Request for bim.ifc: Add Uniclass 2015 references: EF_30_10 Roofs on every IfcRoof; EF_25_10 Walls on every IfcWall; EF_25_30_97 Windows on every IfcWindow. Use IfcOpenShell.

First a look at what the model holds.

```python
import ifcopenshell

model = ifcopenshell.open("bim.ifc")
print(model.schema)
print("classifications:", [c.Name for c in model.by_type("IfcClassification")])
for ifc_class in ("IfcDoor", "IfcRoof", "IfcStair", "IfcWall", "IfcWindow"):
    print(ifc_class, len(model.by_type(ifc_class)))
```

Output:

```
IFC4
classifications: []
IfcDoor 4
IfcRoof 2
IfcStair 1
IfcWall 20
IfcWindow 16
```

```python
import ifcopenshell
import ifcopenshell.api.classification

model = ifcopenshell.open("bim.ifc")

system = ifcopenshell.api.classification.add_classification(model, classification="Uniclass 2015")

codes = {
    "IfcRoof": ("EF_30_10", "Roofs"),
    "IfcWall": ("EF_25_10", "Walls"),
    "IfcWindow": ("EF_25_30_97", "Windows"),
}
for ifc_class, (code, name) in codes.items():
    products = model.by_type(ifc_class)
    ifcopenshell.api.classification.add_reference(
        model, products=products, classification=system, identification=code, name=name
    )
    print(code, len(products))

model.write("bim_rev.ifc")
```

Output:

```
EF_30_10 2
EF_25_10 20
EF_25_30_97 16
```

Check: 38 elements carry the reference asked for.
